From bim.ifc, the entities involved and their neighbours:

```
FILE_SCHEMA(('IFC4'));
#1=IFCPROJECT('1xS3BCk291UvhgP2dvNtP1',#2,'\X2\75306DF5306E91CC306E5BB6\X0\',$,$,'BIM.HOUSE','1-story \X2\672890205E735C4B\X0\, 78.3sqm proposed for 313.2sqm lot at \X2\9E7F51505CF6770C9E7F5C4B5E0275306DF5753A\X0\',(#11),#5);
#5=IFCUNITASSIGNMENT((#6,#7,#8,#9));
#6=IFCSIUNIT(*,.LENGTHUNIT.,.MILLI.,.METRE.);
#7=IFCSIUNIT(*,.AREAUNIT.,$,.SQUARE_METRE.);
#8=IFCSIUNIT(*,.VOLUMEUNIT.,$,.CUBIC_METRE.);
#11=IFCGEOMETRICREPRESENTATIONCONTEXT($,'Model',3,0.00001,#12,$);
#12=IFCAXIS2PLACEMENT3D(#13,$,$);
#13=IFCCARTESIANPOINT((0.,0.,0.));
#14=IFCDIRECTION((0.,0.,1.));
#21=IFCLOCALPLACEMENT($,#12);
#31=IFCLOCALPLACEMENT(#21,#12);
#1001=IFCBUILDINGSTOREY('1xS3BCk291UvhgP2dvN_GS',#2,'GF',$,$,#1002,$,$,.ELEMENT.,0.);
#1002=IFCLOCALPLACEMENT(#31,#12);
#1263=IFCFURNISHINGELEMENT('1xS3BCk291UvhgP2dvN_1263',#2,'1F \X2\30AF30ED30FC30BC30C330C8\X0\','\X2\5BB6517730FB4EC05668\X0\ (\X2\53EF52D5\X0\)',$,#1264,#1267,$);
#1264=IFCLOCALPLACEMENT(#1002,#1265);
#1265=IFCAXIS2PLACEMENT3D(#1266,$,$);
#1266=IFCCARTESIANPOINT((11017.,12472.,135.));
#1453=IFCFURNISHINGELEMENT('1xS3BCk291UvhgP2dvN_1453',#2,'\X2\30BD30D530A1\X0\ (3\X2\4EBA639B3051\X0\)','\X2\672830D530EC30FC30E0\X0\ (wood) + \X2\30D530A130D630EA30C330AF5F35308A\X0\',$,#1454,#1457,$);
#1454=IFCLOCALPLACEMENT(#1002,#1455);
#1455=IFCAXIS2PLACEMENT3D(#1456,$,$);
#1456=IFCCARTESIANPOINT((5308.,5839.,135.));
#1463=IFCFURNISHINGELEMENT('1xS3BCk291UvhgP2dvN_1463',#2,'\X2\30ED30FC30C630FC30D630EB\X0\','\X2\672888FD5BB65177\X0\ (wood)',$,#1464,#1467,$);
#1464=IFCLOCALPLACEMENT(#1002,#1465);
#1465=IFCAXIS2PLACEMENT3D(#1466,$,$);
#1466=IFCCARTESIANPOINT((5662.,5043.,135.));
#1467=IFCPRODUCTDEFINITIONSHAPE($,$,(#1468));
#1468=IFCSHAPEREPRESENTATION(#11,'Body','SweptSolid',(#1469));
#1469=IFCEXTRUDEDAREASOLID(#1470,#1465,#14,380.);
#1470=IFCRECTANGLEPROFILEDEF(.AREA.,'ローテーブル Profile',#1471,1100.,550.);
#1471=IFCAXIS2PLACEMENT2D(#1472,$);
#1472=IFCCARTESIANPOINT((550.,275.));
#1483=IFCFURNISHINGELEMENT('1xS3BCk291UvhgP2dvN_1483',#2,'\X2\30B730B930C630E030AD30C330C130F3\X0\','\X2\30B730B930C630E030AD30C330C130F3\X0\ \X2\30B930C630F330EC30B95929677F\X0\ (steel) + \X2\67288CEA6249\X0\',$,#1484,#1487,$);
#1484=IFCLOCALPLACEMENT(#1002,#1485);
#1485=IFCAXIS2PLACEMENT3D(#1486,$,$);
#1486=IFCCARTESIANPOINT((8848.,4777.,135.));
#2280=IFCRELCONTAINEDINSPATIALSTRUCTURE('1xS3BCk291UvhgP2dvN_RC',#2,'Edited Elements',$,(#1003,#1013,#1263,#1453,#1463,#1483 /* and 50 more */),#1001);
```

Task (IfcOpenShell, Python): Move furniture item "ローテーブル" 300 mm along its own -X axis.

```python
import ifcopenshell
import ifcopenshell.api.geometry
import ifcopenshell.util.placement
import ifcopenshell.util.unit

model = ifcopenshell.open("bim.ifc")
unit_scale = ifcopenshell.util.unit.calculate_unit_scale(model)

item = model.by_guid("1xS3BCk291UvhgP2dvN_1463")
matrix = ifcopenshell.util.placement.get_local_placement(item.ObjectPlacement)
matrix[:3, 3] -= matrix[:3, 0] * 0.3 / unit_scale
ifcopenshell.api.geometry.edit_object_placement(model, product=item, matrix=matrix, is_si=False)

print(ifcopenshell.util.placement.get_local_placement(item.ObjectPlacement).round(3) + 0.0)

model.write("bim_rev.ifc")
```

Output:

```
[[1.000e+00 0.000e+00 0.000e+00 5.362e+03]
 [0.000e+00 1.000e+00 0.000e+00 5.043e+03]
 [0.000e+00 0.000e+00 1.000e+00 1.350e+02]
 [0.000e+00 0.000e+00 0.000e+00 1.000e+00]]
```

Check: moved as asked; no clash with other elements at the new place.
